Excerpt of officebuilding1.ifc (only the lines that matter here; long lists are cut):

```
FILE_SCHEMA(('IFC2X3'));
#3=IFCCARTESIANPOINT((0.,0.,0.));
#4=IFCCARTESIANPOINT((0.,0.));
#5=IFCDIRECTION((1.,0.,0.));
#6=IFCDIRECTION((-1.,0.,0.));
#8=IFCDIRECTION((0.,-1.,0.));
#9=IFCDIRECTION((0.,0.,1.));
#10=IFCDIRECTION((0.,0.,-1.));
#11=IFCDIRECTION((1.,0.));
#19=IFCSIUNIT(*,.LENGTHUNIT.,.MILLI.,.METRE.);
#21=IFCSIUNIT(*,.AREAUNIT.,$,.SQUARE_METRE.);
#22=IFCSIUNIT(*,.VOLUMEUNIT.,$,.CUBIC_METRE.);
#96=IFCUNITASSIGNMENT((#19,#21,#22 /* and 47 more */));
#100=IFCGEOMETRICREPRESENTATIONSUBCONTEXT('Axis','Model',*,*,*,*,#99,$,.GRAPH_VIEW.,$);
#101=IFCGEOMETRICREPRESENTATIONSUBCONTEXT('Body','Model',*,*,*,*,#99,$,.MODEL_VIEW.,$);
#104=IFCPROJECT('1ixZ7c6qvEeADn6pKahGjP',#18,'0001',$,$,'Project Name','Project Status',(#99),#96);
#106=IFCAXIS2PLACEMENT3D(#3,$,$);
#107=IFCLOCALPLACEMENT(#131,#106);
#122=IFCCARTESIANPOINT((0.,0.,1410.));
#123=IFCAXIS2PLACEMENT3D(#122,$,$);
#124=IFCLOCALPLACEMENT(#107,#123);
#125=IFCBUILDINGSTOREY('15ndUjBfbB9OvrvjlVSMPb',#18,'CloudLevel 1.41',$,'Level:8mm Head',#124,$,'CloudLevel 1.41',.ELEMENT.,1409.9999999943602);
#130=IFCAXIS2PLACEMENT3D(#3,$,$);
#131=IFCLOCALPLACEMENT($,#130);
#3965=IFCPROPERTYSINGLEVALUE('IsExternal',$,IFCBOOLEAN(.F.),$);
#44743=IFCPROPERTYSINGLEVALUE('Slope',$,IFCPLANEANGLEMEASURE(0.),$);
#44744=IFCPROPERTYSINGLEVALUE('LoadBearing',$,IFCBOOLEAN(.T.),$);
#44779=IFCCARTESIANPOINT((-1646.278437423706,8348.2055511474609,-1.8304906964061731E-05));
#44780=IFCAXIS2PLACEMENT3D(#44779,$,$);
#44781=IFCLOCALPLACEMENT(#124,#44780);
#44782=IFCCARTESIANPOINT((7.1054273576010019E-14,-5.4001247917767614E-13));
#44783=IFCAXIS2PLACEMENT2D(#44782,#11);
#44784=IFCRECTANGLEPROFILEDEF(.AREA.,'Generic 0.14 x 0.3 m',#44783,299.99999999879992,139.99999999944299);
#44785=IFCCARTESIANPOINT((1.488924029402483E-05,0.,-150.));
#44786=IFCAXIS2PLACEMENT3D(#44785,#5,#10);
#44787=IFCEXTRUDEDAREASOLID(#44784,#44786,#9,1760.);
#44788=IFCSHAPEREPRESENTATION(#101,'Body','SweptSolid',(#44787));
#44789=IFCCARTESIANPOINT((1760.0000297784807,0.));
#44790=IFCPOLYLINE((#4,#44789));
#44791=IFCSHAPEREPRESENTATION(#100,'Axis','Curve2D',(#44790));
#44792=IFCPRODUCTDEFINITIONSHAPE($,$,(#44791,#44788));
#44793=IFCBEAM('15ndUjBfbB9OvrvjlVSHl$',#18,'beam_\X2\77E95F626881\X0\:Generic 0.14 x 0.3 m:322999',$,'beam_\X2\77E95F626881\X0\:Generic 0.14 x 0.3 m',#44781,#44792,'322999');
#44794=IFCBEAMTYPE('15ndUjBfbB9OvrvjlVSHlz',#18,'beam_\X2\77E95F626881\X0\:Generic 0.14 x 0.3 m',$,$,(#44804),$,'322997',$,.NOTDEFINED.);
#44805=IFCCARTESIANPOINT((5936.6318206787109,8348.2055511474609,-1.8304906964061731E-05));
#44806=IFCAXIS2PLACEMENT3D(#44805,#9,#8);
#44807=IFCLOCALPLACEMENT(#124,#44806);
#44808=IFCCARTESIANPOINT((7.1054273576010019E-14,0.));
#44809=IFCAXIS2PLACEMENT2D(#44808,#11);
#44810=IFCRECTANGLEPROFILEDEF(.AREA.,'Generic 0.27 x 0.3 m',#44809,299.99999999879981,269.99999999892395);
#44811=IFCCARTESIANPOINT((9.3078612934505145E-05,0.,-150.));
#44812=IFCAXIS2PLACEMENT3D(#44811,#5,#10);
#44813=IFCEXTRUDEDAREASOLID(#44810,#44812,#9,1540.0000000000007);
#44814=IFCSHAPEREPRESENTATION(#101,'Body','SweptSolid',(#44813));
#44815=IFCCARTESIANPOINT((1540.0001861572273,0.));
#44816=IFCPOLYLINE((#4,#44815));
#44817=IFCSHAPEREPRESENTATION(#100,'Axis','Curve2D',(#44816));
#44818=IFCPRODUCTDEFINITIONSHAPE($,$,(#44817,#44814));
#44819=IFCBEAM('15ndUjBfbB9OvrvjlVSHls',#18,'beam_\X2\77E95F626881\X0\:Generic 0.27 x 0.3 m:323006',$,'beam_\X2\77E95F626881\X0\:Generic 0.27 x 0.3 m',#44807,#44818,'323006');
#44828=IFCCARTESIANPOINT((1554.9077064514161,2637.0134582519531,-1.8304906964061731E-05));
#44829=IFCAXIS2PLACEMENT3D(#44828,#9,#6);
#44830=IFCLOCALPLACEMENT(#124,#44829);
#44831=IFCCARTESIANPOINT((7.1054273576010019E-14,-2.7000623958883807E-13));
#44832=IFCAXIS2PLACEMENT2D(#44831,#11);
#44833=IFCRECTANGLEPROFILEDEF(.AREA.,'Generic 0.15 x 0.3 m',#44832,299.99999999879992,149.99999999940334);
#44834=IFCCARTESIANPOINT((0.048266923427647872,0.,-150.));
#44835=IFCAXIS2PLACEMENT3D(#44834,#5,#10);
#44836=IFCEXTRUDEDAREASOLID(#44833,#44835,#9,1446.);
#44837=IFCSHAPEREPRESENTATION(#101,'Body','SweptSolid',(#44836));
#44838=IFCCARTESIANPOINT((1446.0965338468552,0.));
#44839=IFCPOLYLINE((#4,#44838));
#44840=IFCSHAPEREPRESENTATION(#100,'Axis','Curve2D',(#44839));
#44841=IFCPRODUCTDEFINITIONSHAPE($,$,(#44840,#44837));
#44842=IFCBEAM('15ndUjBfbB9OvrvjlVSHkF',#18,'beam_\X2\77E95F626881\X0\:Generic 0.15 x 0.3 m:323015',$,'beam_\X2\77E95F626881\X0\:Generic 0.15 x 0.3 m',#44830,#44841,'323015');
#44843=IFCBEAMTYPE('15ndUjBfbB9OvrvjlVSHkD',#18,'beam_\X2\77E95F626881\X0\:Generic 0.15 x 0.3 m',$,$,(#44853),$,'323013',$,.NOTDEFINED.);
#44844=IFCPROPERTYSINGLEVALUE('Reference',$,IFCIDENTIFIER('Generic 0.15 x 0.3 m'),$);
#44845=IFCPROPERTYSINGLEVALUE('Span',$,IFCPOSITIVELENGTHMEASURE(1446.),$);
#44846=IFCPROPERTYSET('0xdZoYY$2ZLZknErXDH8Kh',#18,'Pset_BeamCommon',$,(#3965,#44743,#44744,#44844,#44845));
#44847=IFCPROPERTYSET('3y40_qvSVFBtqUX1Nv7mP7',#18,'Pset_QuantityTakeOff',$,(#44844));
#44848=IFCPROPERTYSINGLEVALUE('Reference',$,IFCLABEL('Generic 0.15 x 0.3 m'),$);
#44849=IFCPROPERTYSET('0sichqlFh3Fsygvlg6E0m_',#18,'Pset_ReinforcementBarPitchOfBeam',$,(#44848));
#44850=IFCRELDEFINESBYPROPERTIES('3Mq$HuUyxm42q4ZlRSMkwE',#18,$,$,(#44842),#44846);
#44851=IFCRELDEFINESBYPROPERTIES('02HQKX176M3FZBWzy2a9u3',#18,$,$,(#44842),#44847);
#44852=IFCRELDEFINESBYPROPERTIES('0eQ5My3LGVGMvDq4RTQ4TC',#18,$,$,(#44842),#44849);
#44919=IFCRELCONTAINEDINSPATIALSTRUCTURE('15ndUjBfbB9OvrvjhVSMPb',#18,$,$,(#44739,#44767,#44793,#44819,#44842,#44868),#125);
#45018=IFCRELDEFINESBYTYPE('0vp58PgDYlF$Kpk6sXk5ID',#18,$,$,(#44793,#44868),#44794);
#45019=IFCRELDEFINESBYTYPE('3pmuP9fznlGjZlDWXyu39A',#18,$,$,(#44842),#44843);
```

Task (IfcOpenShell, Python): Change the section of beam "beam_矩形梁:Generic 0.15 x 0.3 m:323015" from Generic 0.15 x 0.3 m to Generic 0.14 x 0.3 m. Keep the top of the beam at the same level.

```python
import ifcopenshell
import ifcopenshell.api.pset
import ifcopenshell.api.type
import ifcopenshell.util.element
import ifcopenshell.util.representation

model = ifcopenshell.open("officebuilding1.ifc")

member = model.by_guid("15ndUjBfbB9OvrvjlVSHkF")
source = next(p for p in model.by_type("IfcRectangleProfileDef") if p.ProfileName == "Generic 0.14 x 0.3 m")

body = ifcopenshell.util.representation.get_representation(member, "Model", "Body")
solid = body.Items[0]
old_profile = solid.SweptArea

# Copy the section's sizes but keep this member's own profile position.
profile = ifcopenshell.util.element.copy(model, source)
# Profiles are centred, so shift by half the change in depth to hold the top.
shift = (old_profile.XDim - profile.XDim) / 2
x, y = old_profile.Position.Location.Coordinates
up = (-1.0, 0.0)  # upwards, in the solid's own plane
location = model.createIfcCartesianPoint((x + up[0] * shift, y + up[1] * shift))
profile.Position = model.createIfcAxis2Placement2D(location, old_profile.Position.RefDirection)
solid.SweptArea = profile
if not model.get_total_inverses(old_profile):
    ifcopenshell.util.element.remove_deep2(model, old_profile)

new_type = model.by_id(44794)
ifcopenshell.api.type.assign_type(
    model, related_objects=[member], relating_type=new_type, should_map_representations=False
)
member.Name = member.Name.replace("Generic 0.15 x 0.3 m", "Generic 0.14 x 0.3 m")
member.ObjectType = "beam_矩形梁:Generic 0.14 x 0.3 m"
pset = model.by_id(ifcopenshell.util.element.get_pset(member, "Pset_BeamCommon", should_inherit=False)["id"])
ifcopenshell.api.pset.edit_pset(model, pset=pset, properties={"Reference": "Generic 0.14 x 0.3 m"})
pset = model.by_id(ifcopenshell.util.element.get_pset(member, "Pset_QuantityTakeOff", should_inherit=False)["id"])
ifcopenshell.api.pset.edit_pset(model, pset=pset, properties={"Reference": "Generic 0.14 x 0.3 m"})
pset = model.by_id(ifcopenshell.util.element.get_pset(member, "Pset_ReinforcementBarPitchOfBeam", should_inherit=False)["id"])
ifcopenshell.api.pset.edit_pset(model, pset=pset, properties={"Reference": "Generic 0.14 x 0.3 m"})

print(solid.SweptArea)

model.write("officebuilding1_v2.ifc")
```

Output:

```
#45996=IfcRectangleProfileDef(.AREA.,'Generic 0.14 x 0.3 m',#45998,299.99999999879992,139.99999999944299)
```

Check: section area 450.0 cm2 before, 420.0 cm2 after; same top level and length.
